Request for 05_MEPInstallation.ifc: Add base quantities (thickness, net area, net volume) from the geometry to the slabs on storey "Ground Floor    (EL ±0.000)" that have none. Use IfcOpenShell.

First a look at what the model holds.

```python
import ifcopenshell
import ifcopenshell.util.element
import ifcopenshell.util.unit

model = ifcopenshell.open("05_MEPInstallation.ifc")
print(model.schema)
for unit_type in ("LENGTHUNIT", "AREAUNIT", "VOLUMEUNIT"):
    print(unit_type, ifcopenshell.util.unit.calculate_unit_scale(model, unit_type))
storey = next(s for s in model.by_type("IfcBuildingStorey") if s.Name == "Ground Floor    (EL ±0.000)")
slabs = [e for e in ifcopenshell.util.element.get_decomposition(storey) if e.is_a("IfcSlab")]
for e in sorted(slabs, key=lambda e: e.id()):
    print(e.id(), e.is_a(), e.Name, list(ifcopenshell.util.element.get_psets(e, qtos_only=True)), sep=" | ")
```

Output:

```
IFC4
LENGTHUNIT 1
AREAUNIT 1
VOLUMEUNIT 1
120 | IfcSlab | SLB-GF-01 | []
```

```python
import ifcopenshell
import ifcopenshell.api.pset
import ifcopenshell.geom
import ifcopenshell.util.element
import ifcopenshell.util.shape
import ifcopenshell.util.unit

model = ifcopenshell.open("05_MEPInstallation.ifc")
unit_scale = ifcopenshell.util.unit.calculate_unit_scale(model)
area_scale = ifcopenshell.util.unit.calculate_unit_scale(model, "AREAUNIT")
volume_scale = ifcopenshell.util.unit.calculate_unit_scale(model, "VOLUMEUNIT")
settings = ifcopenshell.geom.settings()

storey = next(s for s in model.by_type("IfcBuildingStorey") if s.Name == "Ground Floor    (EL ±0.000)")
slabs = [e for e in ifcopenshell.util.element.get_decomposition(storey) if e.is_a("IfcSlab")]

for e in sorted(slabs, key=lambda e: e.id()):
    if ifcopenshell.util.element.get_psets(e, qtos_only=True, should_inherit=False):
        continue
    # Geometry comes back in metres, in the element's own axes.
    shape = ifcopenshell.geom.create_shape(settings, e)
    values = {
        "Width": ifcopenshell.util.shape.get_z(shape.geometry) / unit_scale,
        "NetArea": ifcopenshell.util.shape.get_footprint_area(shape.geometry) / area_scale,
        "NetVolume": ifcopenshell.util.shape.get_volume(shape.geometry) / volume_scale,
    }
    qto = ifcopenshell.api.pset.add_qto(model, product=e, name="Qto_SlabBaseQuantities")
    ifcopenshell.api.pset.edit_qto(model, qto=qto, properties=values)
    print(e.id(), {k: round(v, 3) for k, v in values.items()})

model.write("05_MEPInstallation_edited.ifc")
```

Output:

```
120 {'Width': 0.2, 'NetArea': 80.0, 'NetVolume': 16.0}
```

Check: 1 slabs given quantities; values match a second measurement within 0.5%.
